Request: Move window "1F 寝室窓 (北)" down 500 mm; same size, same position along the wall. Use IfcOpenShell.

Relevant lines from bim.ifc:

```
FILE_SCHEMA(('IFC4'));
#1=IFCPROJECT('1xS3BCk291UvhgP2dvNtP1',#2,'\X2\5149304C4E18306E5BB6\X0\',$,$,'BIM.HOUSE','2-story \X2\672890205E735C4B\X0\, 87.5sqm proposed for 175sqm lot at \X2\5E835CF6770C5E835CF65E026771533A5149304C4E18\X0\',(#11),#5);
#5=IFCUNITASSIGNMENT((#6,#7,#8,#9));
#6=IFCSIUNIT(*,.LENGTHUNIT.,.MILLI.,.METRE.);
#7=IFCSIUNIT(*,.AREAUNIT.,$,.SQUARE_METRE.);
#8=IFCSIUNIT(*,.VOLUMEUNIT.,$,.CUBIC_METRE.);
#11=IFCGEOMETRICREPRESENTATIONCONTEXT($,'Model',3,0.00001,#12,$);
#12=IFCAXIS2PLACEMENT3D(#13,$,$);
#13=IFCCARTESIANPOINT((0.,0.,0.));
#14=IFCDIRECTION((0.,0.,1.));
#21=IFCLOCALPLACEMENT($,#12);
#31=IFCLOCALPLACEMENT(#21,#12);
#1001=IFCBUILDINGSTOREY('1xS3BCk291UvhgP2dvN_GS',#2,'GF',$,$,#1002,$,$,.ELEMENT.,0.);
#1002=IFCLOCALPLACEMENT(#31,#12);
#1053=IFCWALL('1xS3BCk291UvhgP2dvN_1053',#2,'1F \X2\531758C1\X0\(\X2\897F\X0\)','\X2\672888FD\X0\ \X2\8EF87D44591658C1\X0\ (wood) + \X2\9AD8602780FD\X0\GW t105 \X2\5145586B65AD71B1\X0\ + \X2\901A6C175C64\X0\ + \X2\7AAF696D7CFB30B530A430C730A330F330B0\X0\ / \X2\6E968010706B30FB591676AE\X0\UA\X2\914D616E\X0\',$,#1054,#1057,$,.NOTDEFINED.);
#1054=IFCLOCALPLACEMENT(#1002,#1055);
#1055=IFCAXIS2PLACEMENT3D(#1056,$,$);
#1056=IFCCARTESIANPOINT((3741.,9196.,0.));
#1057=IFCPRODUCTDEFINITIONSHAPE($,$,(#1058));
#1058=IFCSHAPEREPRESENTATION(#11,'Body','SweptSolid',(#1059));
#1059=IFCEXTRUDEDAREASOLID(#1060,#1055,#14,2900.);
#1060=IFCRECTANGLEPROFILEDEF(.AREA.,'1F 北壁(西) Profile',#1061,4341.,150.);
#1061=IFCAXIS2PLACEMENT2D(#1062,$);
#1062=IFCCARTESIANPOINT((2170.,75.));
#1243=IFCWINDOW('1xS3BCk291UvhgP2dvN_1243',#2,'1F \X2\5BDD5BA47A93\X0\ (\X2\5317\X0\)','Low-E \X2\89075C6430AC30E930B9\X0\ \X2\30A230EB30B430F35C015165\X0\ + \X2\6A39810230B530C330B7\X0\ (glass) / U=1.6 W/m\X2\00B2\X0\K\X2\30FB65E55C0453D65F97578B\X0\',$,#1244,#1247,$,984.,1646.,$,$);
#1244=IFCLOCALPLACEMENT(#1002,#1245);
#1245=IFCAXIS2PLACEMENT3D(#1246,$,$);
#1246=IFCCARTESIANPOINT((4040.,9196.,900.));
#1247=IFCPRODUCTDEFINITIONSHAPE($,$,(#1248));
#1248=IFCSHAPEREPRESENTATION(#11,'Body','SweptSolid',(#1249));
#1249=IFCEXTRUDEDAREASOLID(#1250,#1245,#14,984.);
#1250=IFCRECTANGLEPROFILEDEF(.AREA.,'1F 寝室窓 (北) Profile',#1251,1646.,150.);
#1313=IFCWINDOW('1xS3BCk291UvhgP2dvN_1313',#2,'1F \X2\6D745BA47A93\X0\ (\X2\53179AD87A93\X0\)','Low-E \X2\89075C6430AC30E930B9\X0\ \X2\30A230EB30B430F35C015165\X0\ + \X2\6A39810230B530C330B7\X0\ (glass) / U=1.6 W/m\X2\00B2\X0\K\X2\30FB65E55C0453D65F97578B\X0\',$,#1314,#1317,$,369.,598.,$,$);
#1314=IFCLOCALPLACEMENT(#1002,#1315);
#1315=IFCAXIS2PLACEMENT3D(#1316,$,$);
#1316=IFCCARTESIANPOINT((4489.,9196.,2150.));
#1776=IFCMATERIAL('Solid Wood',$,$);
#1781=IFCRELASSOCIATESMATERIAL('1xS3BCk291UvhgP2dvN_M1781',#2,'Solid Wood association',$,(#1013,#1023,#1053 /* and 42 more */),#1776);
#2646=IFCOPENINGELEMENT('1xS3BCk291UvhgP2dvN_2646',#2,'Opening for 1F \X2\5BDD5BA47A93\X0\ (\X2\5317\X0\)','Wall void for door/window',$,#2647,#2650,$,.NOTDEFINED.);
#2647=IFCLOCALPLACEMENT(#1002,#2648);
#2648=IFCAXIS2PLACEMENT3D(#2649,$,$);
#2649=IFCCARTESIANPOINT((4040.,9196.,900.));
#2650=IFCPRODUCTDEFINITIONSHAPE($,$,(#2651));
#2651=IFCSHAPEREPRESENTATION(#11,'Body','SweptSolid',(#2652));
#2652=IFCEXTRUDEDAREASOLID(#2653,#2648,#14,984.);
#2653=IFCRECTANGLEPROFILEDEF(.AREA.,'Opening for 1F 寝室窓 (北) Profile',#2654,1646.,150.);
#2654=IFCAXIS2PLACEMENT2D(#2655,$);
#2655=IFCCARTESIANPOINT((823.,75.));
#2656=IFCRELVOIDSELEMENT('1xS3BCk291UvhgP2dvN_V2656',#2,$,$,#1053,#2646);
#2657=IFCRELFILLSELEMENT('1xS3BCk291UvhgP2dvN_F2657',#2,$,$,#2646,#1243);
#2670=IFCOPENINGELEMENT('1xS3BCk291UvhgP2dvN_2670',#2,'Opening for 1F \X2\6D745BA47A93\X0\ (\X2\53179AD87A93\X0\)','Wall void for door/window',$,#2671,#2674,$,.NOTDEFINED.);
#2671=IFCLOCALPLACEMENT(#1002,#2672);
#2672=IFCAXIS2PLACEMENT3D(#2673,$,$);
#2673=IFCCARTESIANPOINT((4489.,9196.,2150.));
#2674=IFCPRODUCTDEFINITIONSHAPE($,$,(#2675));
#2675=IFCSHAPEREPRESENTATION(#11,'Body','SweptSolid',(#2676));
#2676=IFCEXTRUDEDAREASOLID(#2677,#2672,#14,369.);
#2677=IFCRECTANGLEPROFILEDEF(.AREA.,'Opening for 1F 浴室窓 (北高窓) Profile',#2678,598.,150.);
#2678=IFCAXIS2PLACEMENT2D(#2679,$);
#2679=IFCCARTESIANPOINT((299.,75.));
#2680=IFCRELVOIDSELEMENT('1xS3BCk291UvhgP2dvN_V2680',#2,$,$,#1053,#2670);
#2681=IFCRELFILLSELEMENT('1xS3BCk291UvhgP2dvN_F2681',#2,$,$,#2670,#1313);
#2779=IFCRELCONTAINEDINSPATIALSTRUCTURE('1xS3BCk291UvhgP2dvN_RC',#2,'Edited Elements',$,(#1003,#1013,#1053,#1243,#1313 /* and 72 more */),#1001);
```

```python
import numpy as np
import ifcopenshell
import ifcopenshell.api.geometry
import ifcopenshell.util.placement
import ifcopenshell.util.unit

model = ifcopenshell.open("bim.ifc")
unit_scale = ifcopenshell.util.unit.calculate_unit_scale(model)

window = model.by_guid("1xS3BCk291UvhgP2dvN_1243")
opening = window.FillsVoids[0].RelatingOpeningElement
dz = -500.0

shift = np.array([0.0, 0.0, dz])
# The window is not placed relative to its opening, so move both.
for product in (opening, window):
    matrix = ifcopenshell.util.placement.get_local_placement(product.ObjectPlacement)
    matrix[:3, 3] += shift
    ifcopenshell.api.geometry.edit_object_placement(model, product=product, matrix=matrix, is_si=False)

print(f"moved by {dz * unit_scale:+.3f} m")

model.write("bim_updated.ifc")
```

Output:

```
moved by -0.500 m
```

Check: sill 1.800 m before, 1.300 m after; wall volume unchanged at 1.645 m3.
